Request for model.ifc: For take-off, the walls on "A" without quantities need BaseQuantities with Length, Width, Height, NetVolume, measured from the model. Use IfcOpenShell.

First a look at what the model holds.

```python
import ifcopenshell
import ifcopenshell.util.element
import ifcopenshell.util.unit

model = ifcopenshell.open("model.ifc")
print(model.schema)
for unit_type in ("LENGTHUNIT", "AREAUNIT", "VOLUMEUNIT"):
    print(unit_type, ifcopenshell.util.unit.calculate_unit_scale(model, unit_type))
storey = next(s for s in model.by_type("IfcBuildingStorey") if s.Name == "A")
walls = [e for e in ifcopenshell.util.element.get_decomposition(storey) if e.is_a("IfcWall")]
for e in sorted(walls, key=lambda e: e.id()):
    print(e.id(), e.is_a(), e.Name, list(ifcopenshell.util.element.get_psets(e, qtos_only=True)), sep=" | ")
```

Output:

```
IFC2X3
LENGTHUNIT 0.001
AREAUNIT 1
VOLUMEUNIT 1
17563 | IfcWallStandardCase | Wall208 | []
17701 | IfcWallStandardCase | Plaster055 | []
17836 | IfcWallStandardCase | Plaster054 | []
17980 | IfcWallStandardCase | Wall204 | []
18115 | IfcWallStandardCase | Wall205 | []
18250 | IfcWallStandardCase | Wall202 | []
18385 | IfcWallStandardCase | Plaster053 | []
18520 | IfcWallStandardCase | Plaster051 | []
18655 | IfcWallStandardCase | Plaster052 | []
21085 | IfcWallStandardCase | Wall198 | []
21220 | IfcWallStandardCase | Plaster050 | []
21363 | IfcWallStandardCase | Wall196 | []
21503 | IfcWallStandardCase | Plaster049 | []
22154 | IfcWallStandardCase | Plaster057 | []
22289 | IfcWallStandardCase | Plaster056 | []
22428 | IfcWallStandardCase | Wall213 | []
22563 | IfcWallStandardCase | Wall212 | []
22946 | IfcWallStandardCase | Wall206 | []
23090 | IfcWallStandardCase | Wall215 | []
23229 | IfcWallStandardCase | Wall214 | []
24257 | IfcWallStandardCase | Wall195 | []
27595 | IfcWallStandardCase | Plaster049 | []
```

```python
import ifcopenshell
import ifcopenshell.api.pset
import ifcopenshell.geom
import ifcopenshell.util.element
import ifcopenshell.util.shape
import ifcopenshell.util.unit

model = ifcopenshell.open("model.ifc")
unit_scale = ifcopenshell.util.unit.calculate_unit_scale(model)
volume_scale = ifcopenshell.util.unit.calculate_unit_scale(model, "VOLUMEUNIT")
settings = ifcopenshell.geom.settings()

storey = next(s for s in model.by_type("IfcBuildingStorey") if s.Name == "A")
walls = [e for e in ifcopenshell.util.element.get_decomposition(storey) if e.is_a("IfcWall")]

for e in sorted(walls, key=lambda e: e.id()):
    if ifcopenshell.util.element.get_psets(e, qtos_only=True, should_inherit=False):
        continue
    # Geometry comes back in metres, in the element's own axes.
    shape = ifcopenshell.geom.create_shape(settings, e)
    values = {
        "Length": ifcopenshell.util.shape.get_x(shape.geometry) / unit_scale,
        "Width": ifcopenshell.util.shape.get_y(shape.geometry) / unit_scale,
        "Height": ifcopenshell.util.shape.get_z(shape.geometry) / unit_scale,
        "NetVolume": ifcopenshell.util.shape.get_volume(shape.geometry) / volume_scale,
    }
    qto = ifcopenshell.api.pset.add_qto(model, product=e, name="BaseQuantities")
    ifcopenshell.api.pset.edit_qto(model, qto=qto, properties=values)
    print(e.id(), {k: round(v, 3) for k, v in values.items()})

model.write("model_v2.ifc")
```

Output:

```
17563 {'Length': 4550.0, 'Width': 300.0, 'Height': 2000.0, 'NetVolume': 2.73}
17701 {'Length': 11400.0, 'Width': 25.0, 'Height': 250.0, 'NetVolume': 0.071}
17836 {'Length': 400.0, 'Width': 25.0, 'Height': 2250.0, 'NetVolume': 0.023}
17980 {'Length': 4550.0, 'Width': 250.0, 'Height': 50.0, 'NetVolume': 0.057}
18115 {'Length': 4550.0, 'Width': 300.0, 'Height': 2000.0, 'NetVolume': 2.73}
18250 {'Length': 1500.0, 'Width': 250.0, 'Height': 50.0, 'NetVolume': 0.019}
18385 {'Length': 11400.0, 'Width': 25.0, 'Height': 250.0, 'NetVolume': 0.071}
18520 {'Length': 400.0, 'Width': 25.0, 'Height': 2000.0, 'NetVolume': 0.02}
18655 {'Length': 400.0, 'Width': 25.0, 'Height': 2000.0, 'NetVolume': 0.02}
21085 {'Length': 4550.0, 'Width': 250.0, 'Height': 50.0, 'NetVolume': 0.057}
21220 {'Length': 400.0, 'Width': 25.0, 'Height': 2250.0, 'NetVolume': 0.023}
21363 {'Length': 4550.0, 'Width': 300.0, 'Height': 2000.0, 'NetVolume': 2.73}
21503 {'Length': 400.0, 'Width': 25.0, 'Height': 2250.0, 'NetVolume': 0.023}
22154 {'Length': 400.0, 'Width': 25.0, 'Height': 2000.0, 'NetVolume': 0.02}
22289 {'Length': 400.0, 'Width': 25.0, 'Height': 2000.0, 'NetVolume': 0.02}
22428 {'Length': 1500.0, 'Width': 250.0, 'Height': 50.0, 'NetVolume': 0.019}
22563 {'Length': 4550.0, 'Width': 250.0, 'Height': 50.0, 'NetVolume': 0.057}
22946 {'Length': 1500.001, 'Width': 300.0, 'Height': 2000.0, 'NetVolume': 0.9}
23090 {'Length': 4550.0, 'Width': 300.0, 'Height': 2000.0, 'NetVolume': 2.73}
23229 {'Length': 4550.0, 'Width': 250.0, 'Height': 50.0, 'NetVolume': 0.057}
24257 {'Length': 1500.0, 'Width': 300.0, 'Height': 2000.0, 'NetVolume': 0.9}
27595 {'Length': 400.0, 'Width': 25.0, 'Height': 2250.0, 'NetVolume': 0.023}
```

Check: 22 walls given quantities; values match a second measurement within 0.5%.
